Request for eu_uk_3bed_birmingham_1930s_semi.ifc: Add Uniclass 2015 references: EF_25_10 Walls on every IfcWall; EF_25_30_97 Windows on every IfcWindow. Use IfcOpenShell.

First a look at what the model holds.

```python
import ifcopenshell

model = ifcopenshell.open("eu_uk_3bed_birmingham_1930s_semi.ifc")
print(model.schema)
print("classifications:", [c.Name for c in model.by_type("IfcClassification")])
for ifc_class in ("IfcDoor", "IfcRoof", "IfcStair", "IfcWall", "IfcWindow"):
    print(ifc_class, len(model.by_type(ifc_class)))
```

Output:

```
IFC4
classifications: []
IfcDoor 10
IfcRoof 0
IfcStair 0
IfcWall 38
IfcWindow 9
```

```python
import ifcopenshell
import ifcopenshell.api.classification

model = ifcopenshell.open("eu_uk_3bed_birmingham_1930s_semi.ifc")

system = ifcopenshell.api.classification.add_classification(model, classification="Uniclass 2015")

codes = {
    "IfcWall": ("EF_25_10", "Walls"),
    "IfcWindow": ("EF_25_30_97", "Windows"),
}
for ifc_class, (code, name) in codes.items():
    products = model.by_type(ifc_class)
    ifcopenshell.api.classification.add_reference(
        model, products=products, classification=system, identification=code, name=name
    )
    print(code, len(products))

model.write("eu_uk_3bed_birmingham_1930s_semi_updated.ifc")
```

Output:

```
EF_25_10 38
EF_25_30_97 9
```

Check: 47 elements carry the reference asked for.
